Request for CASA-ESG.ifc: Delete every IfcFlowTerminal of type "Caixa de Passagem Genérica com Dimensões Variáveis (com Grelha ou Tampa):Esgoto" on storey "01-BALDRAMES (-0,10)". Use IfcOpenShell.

First a look at what the model holds.

```python
import ifcopenshell
import ifcopenshell.util.element

model = ifcopenshell.open("CASA-ESG.ifc")
print(model.schema)
storey = next(s for s in model.by_type("IfcBuildingStorey") if s.Name == "01-BALDRAMES (-0,10)")
terminals = [e for e in ifcopenshell.util.element.get_decomposition(storey) if e.is_a("IfcFlowTerminal")]
seen = {}
for e in terminals:
    element_type = ifcopenshell.util.element.get_type(e)
    name = element_type.Name if element_type not in (None, e) else None
    seen[name] = seen.get(name, 0) + 1
for name, count in sorted(seen.items(), key=str):
    print(count, "x", name)
```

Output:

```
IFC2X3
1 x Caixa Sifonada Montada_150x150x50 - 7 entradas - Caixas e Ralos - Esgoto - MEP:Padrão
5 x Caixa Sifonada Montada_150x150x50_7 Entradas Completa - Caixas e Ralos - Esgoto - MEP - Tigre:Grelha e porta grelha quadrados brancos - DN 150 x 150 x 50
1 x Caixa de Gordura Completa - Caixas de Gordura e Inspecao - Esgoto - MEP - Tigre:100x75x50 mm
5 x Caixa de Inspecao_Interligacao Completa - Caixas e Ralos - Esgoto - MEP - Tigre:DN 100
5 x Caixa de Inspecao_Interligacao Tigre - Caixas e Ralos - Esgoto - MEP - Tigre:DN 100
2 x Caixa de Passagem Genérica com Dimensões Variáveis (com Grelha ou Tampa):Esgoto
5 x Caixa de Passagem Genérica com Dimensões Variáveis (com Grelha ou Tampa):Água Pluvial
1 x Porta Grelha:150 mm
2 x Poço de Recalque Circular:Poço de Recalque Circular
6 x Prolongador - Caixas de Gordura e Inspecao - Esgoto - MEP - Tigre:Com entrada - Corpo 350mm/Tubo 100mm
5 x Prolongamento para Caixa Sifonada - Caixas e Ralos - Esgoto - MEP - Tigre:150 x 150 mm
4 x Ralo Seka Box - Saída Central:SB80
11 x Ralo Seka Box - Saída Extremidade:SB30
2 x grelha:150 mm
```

```python
import ifcopenshell
import ifcopenshell.api.root
import ifcopenshell.util.element

model = ifcopenshell.open("CASA-ESG.ifc")

storey = next(s for s in model.by_type("IfcBuildingStorey") if s.Name == "01-BALDRAMES (-0,10)")
terminals = [e for e in ifcopenshell.util.element.get_decomposition(storey) if e.is_a("IfcFlowTerminal")]
targets = [e for e in terminals if (t := ifcopenshell.util.element.get_type(e)) not in (None, e) and t.Name == "Caixa de Passagem Genérica com Dimensões Variáveis (com Grelha ou Tampa):Esgoto"]

for e in targets:
    ifcopenshell.api.root.remove_product(model, product=e)
print(len(targets), "removed")

model.write("CASA-ESG_v2.ifc")
```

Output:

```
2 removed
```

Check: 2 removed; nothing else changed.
